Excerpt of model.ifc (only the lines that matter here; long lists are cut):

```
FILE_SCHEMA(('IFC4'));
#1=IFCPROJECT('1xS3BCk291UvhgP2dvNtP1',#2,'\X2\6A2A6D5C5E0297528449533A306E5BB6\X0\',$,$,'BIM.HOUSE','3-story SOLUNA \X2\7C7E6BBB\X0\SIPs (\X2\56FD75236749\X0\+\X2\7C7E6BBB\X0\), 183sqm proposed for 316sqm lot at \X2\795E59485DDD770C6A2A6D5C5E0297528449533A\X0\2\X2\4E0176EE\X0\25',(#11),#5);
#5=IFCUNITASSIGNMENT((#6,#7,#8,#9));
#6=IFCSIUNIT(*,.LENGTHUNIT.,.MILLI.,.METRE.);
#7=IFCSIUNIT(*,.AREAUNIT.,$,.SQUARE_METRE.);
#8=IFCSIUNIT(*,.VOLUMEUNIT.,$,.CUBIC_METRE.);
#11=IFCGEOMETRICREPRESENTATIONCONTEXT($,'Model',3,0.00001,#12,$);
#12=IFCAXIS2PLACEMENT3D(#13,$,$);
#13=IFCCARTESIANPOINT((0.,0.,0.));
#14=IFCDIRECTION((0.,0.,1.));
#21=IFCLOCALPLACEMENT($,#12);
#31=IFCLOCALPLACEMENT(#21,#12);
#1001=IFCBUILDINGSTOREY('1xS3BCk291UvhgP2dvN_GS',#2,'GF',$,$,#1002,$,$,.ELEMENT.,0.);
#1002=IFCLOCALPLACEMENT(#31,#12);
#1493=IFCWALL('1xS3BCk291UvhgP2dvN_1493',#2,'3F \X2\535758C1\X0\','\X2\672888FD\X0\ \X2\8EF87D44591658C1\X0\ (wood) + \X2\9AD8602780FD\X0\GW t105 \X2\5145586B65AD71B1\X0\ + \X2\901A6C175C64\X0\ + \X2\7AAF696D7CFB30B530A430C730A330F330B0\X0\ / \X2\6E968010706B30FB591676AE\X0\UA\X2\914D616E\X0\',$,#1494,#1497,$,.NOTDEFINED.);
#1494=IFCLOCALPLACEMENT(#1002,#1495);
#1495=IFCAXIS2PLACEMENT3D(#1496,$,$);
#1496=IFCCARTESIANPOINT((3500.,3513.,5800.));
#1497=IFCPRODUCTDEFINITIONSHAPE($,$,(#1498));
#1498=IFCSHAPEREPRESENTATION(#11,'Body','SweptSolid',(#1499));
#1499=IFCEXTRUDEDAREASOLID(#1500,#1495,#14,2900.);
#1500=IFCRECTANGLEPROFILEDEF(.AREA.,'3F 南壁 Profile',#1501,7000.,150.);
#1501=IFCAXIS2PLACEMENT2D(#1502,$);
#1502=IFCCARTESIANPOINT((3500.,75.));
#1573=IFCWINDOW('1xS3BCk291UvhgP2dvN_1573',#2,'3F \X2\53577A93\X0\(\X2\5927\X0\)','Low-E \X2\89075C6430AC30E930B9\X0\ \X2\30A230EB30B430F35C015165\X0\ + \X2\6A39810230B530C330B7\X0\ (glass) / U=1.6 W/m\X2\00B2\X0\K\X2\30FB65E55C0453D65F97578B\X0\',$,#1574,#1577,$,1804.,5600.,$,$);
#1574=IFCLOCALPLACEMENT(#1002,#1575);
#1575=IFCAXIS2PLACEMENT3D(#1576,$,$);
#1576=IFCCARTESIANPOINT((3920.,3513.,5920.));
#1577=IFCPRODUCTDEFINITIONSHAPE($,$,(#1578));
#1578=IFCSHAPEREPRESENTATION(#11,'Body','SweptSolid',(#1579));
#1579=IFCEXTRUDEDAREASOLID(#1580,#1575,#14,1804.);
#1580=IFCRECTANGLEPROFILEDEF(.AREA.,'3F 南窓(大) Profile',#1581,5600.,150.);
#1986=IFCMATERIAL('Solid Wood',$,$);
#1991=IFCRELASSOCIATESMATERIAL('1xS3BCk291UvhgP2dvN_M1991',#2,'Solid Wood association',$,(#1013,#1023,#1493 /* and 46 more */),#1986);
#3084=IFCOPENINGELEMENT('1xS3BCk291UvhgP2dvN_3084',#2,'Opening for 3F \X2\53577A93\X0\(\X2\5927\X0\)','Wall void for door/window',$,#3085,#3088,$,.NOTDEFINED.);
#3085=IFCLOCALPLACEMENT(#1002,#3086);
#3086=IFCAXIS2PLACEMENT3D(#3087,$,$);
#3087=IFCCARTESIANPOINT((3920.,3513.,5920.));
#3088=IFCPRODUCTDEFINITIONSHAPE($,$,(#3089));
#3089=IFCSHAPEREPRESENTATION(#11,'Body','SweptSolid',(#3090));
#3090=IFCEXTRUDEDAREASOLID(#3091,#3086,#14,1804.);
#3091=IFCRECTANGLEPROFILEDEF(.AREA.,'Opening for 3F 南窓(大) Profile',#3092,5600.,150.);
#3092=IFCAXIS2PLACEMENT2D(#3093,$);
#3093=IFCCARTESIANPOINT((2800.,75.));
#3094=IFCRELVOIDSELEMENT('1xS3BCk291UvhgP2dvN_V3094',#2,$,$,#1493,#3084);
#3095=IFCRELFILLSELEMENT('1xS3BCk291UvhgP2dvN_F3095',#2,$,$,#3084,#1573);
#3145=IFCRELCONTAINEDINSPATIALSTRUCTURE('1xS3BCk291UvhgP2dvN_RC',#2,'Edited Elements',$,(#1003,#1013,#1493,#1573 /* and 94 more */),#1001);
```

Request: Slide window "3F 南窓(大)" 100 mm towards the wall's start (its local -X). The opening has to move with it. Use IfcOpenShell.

```python
import ifcopenshell
import ifcopenshell.api.geometry
import ifcopenshell.util.placement

model = ifcopenshell.open("model.ifc")

window = model.by_guid("1xS3BCk291UvhgP2dvN_1573")
opening = window.FillsVoids[0].RelatingOpeningElement
wall = opening.VoidsElements[0].RelatingBuildingElement

wall_matrix = ifcopenshell.util.placement.get_local_placement(wall.ObjectPlacement)
shift = wall_matrix[:3, 0] * -100.0
before = ifcopenshell.util.placement.get_local_placement(window.ObjectPlacement)[:3, 3].copy()

# The window is not placed relative to its opening, so move both.
for product in (opening, window):
    matrix = ifcopenshell.util.placement.get_local_placement(product.ObjectPlacement)
    matrix[:3, 3] += shift
    ifcopenshell.api.geometry.edit_object_placement(model, product=product, matrix=matrix, is_si=False)

after = ifcopenshell.util.placement.get_local_placement(window.ObjectPlacement)[:3, 3]
print("window moved by", (after - before).round(3) + 0.0)

model.write("model-out.ifc")
```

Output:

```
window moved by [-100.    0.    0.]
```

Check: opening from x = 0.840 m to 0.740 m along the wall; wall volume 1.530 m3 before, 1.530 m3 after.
